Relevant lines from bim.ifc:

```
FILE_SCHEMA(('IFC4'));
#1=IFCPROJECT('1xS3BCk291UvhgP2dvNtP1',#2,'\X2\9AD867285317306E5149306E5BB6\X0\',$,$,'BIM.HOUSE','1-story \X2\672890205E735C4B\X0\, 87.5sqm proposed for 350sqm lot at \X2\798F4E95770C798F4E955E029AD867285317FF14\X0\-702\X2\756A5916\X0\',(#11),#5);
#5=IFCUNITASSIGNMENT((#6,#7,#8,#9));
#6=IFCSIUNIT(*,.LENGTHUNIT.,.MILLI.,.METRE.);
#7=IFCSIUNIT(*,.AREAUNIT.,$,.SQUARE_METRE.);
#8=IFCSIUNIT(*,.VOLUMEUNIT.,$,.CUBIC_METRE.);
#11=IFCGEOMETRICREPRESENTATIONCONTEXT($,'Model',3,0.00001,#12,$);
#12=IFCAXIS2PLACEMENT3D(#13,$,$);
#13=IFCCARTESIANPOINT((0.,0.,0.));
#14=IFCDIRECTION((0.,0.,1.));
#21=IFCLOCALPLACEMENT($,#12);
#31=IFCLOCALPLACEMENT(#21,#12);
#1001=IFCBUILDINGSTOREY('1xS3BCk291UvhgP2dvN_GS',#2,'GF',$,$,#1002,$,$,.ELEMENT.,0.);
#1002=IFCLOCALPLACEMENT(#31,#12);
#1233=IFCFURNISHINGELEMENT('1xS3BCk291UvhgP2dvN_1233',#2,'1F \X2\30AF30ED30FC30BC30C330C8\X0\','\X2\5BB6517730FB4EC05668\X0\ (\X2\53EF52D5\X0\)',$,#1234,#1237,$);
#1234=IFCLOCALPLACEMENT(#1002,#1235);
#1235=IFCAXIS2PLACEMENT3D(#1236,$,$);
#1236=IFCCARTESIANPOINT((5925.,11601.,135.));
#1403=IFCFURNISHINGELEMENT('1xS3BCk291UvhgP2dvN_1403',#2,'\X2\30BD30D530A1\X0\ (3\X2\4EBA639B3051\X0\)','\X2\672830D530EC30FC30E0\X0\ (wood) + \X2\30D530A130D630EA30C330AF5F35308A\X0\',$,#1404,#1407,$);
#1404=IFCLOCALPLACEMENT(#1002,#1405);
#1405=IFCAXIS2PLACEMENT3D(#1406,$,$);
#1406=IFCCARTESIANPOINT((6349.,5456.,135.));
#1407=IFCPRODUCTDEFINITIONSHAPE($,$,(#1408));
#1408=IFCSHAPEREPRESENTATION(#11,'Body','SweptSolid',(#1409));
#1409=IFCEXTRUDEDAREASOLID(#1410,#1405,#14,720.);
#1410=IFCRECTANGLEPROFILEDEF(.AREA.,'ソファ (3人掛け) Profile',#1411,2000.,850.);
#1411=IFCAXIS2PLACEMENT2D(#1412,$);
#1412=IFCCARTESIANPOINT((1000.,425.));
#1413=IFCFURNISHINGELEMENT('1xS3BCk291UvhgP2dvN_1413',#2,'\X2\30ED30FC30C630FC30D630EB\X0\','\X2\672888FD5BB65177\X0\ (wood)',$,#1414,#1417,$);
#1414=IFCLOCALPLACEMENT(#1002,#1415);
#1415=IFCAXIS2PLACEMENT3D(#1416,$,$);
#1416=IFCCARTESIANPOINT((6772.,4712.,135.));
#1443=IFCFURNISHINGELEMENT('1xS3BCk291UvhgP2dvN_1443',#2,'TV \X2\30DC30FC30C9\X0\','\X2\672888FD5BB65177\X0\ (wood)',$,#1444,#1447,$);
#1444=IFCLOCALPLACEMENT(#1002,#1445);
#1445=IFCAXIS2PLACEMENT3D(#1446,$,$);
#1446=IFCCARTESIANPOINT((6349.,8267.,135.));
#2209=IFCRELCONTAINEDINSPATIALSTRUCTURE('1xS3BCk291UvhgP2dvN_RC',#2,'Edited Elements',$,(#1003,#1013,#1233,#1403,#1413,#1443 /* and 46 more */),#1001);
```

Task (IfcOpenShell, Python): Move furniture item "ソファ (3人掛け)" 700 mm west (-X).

```python
import ifcopenshell
import ifcopenshell.api.geometry
import ifcopenshell.util.placement

model = ifcopenshell.open("bim.ifc")

item = model.by_id(1403)
matrix = ifcopenshell.util.placement.get_local_placement(item.ObjectPlacement)
matrix[0, 3] -= 700.0
ifcopenshell.api.geometry.edit_object_placement(model, product=item, matrix=matrix, is_si=False)

print(ifcopenshell.util.placement.get_local_placement(item.ObjectPlacement).round(3) + 0.0)

model.write("bim_updated.ifc")
```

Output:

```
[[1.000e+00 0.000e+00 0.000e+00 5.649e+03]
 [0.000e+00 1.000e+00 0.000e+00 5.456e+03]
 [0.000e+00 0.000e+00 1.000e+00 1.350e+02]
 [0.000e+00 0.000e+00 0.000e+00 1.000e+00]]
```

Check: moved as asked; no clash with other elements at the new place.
